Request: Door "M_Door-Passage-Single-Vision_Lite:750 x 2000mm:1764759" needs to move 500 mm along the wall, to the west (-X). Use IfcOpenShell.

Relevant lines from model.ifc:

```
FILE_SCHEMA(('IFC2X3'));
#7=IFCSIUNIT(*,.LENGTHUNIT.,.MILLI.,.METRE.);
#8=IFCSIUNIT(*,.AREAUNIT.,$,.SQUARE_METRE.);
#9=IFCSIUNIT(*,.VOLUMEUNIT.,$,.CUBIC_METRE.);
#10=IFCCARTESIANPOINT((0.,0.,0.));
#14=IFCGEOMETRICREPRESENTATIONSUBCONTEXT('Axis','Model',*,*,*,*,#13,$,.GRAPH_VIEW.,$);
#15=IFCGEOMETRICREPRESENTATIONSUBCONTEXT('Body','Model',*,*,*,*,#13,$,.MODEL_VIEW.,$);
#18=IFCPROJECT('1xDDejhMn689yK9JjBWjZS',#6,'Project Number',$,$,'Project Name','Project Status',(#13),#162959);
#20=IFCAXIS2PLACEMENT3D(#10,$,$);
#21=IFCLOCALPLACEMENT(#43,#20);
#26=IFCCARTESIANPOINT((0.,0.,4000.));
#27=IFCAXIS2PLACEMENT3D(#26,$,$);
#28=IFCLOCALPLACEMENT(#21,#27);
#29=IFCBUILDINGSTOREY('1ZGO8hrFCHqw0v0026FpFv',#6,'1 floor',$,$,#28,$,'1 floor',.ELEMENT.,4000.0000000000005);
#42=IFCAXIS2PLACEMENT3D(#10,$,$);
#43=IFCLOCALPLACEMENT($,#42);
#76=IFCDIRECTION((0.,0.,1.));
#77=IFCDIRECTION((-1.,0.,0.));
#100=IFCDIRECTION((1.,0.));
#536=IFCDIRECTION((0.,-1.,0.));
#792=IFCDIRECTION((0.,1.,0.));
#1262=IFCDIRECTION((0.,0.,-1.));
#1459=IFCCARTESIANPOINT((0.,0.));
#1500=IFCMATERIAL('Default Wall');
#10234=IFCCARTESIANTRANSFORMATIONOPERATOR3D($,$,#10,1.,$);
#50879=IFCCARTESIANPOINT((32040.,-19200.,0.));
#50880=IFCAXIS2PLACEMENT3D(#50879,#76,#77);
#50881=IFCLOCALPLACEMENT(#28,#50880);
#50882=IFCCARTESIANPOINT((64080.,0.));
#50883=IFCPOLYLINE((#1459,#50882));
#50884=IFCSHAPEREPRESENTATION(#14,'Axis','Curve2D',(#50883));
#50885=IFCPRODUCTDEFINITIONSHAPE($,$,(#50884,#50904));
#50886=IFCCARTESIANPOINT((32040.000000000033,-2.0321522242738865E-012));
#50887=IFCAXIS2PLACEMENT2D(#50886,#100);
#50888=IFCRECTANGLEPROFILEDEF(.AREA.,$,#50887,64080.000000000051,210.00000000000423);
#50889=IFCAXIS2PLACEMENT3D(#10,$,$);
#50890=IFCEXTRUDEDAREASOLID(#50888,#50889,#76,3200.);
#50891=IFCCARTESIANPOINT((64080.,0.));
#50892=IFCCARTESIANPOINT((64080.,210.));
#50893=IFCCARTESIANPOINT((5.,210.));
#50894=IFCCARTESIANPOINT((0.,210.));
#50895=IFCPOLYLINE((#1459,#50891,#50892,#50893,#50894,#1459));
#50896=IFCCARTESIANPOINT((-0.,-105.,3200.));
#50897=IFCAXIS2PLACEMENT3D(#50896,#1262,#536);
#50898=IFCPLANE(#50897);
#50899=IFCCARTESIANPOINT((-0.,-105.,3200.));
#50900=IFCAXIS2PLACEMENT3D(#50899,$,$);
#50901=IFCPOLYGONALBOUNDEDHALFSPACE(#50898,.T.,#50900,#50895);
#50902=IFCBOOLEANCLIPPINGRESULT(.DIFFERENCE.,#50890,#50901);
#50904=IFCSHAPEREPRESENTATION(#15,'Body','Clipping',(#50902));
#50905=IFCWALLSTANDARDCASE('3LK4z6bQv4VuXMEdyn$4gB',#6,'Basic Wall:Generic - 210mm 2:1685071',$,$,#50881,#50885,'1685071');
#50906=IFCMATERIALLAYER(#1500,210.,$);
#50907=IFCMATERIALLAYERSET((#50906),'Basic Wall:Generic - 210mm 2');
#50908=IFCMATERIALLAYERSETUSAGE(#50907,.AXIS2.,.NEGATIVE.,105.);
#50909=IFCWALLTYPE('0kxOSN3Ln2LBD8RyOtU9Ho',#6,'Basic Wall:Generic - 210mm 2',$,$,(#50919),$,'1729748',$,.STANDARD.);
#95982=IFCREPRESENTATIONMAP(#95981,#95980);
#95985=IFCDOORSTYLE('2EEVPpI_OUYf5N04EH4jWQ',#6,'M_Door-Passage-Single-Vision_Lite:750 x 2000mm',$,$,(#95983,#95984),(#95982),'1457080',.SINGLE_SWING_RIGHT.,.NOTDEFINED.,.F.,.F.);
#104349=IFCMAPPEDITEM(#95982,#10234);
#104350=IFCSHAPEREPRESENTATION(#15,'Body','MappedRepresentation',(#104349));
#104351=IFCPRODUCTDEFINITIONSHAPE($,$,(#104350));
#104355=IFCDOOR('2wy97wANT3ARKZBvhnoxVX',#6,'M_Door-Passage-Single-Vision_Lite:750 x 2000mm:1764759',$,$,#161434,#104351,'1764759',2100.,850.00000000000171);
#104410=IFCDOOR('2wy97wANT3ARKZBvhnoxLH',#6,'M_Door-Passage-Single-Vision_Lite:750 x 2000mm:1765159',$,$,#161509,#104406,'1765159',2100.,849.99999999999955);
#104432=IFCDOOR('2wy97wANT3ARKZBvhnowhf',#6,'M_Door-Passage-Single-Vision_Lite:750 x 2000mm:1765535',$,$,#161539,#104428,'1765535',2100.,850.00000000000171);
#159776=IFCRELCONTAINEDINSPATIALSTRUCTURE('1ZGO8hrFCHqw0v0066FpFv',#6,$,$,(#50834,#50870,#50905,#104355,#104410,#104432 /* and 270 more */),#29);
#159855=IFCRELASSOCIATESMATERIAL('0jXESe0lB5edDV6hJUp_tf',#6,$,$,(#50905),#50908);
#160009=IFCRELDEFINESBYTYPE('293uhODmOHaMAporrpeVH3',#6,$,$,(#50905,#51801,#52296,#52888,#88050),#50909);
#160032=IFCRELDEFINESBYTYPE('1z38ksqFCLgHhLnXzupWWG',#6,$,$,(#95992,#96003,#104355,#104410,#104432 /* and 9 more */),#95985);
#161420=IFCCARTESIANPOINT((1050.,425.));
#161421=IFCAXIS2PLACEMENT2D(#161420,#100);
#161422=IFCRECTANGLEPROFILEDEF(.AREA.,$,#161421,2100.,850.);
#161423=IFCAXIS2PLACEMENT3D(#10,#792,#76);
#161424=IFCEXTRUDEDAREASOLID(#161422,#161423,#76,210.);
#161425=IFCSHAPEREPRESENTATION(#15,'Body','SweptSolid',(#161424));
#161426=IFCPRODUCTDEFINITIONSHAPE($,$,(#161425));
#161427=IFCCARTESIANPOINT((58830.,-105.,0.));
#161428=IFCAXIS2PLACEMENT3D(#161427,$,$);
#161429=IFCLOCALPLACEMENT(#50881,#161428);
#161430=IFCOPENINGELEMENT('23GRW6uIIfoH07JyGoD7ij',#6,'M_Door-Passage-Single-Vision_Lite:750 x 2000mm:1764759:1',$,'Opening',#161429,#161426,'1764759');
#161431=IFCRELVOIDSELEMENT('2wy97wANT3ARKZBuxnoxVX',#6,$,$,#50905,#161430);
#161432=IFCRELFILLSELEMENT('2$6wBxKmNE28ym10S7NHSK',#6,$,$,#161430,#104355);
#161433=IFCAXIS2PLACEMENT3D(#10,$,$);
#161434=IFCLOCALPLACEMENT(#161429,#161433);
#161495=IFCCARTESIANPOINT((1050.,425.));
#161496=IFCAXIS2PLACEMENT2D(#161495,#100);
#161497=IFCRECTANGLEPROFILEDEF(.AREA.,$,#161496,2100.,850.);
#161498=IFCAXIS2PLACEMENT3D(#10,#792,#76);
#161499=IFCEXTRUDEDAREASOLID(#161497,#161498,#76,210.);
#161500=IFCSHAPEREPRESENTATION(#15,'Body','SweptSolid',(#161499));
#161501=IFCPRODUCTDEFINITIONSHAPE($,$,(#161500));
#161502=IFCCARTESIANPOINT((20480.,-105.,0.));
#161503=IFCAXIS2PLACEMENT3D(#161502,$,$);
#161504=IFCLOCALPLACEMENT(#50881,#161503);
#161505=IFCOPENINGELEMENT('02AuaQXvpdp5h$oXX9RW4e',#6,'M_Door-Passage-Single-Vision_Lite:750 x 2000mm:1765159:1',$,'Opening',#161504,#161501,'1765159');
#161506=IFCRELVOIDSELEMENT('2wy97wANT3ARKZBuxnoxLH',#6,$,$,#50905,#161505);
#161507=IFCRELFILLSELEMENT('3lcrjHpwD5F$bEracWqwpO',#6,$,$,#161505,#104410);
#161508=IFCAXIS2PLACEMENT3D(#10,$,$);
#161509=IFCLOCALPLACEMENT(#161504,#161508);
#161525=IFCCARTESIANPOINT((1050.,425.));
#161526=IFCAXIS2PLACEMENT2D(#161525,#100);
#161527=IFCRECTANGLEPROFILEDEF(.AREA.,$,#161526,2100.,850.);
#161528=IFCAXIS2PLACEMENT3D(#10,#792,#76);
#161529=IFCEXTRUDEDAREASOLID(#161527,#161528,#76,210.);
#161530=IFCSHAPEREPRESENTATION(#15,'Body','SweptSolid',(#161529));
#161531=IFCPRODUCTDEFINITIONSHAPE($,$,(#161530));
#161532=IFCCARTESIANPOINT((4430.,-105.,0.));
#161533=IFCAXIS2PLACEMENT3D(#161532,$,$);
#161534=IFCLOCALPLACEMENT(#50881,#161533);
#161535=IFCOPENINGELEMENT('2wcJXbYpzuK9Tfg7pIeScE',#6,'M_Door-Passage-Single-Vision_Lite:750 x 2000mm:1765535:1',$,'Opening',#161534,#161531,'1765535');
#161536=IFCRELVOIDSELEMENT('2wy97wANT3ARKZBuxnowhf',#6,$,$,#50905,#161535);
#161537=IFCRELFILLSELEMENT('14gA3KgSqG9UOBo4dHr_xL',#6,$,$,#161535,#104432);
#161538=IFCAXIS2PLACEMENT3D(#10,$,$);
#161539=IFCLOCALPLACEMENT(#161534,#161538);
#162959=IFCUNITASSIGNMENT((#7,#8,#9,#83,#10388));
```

```python
import ifcopenshell
import ifcopenshell.api.geometry
import ifcopenshell.util.placement
import ifcopenshell.util.unit

model = ifcopenshell.open("model.ifc")
unit_scale = ifcopenshell.util.unit.calculate_unit_scale(model)

door = model.by_guid("2wy97wANT3ARKZBvhnoxVX")
opening = door.FillsVoids[0].RelatingOpeningElement
wall = opening.VoidsElements[0].RelatingBuildingElement

wall_matrix = ifcopenshell.util.placement.get_local_placement(wall.ObjectPlacement)
shift = wall_matrix[:3, 0] * 0.5 / unit_scale
before = ifcopenshell.util.placement.get_local_placement(door.ObjectPlacement)[:3, 3].copy()

# The door is placed relative to its opening, so it follows when the opening moves.
matrix = ifcopenshell.util.placement.get_local_placement(opening.ObjectPlacement)
matrix[:3, 3] += shift
ifcopenshell.api.geometry.edit_object_placement(
    model, product=opening, matrix=matrix, is_si=False, should_transform_children=True
)

after = ifcopenshell.util.placement.get_local_placement(door.ObjectPlacement)[:3, 3]
print("door moved by", (after - before).round(3) + 0.0)

model.write("model-out.ifc")
```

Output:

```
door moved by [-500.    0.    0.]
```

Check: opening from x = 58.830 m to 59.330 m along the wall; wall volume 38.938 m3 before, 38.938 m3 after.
